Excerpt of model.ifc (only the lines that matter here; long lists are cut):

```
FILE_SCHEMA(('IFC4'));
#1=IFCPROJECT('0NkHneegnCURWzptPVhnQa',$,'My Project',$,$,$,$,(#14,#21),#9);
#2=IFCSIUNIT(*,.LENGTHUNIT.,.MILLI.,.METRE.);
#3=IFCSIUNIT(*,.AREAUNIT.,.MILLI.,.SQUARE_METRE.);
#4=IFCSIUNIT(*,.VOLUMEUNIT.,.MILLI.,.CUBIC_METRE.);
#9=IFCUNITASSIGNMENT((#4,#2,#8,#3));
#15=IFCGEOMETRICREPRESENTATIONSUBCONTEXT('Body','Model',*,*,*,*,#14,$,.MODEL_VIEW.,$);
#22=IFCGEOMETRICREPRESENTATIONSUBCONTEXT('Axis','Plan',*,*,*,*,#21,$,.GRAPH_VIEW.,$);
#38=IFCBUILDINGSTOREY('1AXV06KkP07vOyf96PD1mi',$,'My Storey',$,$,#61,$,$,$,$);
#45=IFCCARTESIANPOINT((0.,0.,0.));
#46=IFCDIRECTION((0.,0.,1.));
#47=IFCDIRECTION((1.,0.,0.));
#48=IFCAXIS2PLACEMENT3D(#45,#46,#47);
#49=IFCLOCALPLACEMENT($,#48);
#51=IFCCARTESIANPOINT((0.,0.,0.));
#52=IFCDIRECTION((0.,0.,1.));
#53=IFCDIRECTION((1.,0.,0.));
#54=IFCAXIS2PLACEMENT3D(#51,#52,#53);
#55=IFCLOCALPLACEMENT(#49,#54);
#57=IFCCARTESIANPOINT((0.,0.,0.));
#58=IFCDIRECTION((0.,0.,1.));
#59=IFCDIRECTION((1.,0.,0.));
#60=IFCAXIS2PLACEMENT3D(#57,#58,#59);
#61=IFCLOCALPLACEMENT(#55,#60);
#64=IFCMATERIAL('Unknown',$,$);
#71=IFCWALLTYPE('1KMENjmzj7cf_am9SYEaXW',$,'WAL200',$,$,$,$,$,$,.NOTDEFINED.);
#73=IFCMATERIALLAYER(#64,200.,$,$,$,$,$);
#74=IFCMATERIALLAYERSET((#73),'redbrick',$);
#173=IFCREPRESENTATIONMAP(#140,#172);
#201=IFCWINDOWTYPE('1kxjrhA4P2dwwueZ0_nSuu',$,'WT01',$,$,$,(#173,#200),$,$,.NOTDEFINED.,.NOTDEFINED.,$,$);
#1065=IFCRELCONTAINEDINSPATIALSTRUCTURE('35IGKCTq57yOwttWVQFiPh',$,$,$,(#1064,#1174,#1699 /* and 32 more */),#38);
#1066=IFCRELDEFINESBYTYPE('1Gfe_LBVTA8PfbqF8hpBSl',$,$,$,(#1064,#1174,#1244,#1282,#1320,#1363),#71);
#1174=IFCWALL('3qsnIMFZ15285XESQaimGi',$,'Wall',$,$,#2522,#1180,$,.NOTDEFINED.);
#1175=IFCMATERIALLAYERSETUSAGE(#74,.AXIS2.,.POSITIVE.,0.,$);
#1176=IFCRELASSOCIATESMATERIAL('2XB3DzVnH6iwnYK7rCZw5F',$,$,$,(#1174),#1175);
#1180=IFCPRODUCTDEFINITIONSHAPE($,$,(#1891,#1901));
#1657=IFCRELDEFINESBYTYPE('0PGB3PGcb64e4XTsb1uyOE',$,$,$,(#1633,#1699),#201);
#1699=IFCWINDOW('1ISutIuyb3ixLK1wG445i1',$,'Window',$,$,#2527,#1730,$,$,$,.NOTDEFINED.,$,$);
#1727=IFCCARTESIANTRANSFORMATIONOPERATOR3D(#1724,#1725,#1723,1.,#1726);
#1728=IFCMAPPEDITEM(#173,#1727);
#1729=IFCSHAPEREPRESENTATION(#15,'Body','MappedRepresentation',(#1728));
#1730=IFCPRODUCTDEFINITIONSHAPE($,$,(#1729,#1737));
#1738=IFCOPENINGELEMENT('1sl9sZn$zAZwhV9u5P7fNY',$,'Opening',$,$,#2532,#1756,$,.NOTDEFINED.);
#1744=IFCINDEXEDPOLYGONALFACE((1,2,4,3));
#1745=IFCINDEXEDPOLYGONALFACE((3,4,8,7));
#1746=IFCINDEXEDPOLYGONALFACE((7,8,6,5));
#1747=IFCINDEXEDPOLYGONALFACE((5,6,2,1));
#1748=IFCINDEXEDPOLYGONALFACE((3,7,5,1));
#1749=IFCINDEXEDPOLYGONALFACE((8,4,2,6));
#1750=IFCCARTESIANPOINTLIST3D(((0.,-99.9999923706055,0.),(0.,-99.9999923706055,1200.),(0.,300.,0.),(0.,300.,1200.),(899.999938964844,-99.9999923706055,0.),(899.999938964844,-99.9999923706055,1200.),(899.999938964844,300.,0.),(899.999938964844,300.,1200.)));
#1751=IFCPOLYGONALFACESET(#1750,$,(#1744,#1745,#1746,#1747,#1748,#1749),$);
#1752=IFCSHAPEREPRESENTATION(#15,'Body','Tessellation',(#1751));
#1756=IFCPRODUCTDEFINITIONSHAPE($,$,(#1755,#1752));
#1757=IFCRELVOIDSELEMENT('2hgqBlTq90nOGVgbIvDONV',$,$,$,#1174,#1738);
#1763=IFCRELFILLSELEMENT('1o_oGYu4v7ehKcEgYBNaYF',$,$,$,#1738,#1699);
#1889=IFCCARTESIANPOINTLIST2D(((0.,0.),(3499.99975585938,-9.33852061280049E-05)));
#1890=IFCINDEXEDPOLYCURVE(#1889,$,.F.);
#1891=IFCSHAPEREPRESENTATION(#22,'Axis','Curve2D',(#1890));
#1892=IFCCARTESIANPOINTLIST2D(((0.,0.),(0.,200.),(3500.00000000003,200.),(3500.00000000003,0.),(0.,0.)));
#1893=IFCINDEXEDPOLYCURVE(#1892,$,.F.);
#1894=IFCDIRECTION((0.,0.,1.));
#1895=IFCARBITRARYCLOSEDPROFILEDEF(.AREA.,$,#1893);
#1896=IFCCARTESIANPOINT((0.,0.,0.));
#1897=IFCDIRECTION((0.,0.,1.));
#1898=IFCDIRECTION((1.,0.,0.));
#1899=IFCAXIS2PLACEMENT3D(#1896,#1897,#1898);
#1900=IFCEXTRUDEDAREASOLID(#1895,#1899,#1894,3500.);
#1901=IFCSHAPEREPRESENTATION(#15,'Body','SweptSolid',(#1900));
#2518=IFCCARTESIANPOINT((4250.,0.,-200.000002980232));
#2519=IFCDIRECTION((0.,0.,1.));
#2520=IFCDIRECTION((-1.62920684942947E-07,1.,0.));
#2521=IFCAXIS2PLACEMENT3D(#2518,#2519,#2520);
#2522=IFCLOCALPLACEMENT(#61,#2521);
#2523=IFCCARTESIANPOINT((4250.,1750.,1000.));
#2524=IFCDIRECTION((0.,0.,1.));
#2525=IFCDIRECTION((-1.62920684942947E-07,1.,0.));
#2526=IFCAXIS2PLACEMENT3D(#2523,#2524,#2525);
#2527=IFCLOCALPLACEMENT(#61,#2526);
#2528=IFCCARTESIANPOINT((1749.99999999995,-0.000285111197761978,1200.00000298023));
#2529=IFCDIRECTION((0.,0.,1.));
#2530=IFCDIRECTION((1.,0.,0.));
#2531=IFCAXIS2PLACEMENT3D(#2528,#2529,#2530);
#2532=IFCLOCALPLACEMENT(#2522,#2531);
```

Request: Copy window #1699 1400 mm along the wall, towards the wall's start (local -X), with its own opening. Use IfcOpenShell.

```python
import ifcopenshell
import ifcopenshell.api.feature
import ifcopenshell.api.geometry
import ifcopenshell.api.root
import ifcopenshell.geom
import ifcopenshell.util.element
import ifcopenshell.util.placement
import ifcopenshell.util.shape

model = ifcopenshell.open("model.ifc")
settings = ifcopenshell.geom.settings()


def volume(element):
    """Net volume in cubic metres, openings subtracted."""
    shape = ifcopenshell.geom.create_shape(settings, element)
    return ifcopenshell.util.shape.get_volume(shape.geometry)


window = model.by_guid("1ISutIuyb3ixLK1wG445i1")
opening = window.FillsVoids[0].RelatingOpeningElement
wall = opening.VoidsElements[0].RelatingBuildingElement
before = volume(wall)
shift = ifcopenshell.util.placement.get_local_placement(wall.ObjectPlacement)[:3, 0] * -1400.0

# copy_class copies the void relationship, type, container and properties, but no geometry.
new_opening = ifcopenshell.api.root.copy_class(model, product=opening)
new_opening.Representation = ifcopenshell.util.element.copy_deep(
    model, opening.Representation, exclude=["IfcGeometricRepresentationContext", "IfcRepresentationMap"]
)
new_window = ifcopenshell.api.root.copy_class(model, product=window)
new_window.Representation = ifcopenshell.util.element.copy_deep(
    model, window.Representation, exclude=["IfcGeometricRepresentationContext", "IfcRepresentationMap"]
)
ifcopenshell.api.feature.add_filling(model, opening=new_opening, element=new_window)

for old, new in ((opening, new_opening), (window, new_window)):
    matrix = ifcopenshell.util.placement.get_local_placement(old.ObjectPlacement)
    matrix[:3, 3] += shift
    ifcopenshell.api.geometry.edit_object_placement(model, product=new, matrix=matrix, is_si=False)

after = volume(wall)

print(f"wall volume {before:.3f} -> {after:.3f} m3")

model.write("model_v2.ifc")
```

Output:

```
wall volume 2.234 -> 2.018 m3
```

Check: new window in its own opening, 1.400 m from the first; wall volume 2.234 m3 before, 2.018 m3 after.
